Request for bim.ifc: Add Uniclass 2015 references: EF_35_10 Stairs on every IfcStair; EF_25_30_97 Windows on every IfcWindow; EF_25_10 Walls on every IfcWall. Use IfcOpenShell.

First a look at what the model holds.

```python
import ifcopenshell

model = ifcopenshell.open("bim.ifc")
print(model.schema)
print("classifications:", [c.Name for c in model.by_type("IfcClassification")])
for ifc_class in ("IfcDoor", "IfcRoof", "IfcStair", "IfcWall", "IfcWindow"):
    print(ifc_class, len(model.by_type(ifc_class)))
```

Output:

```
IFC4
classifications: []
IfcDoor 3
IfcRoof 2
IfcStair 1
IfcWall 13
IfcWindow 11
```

```python
import ifcopenshell
import ifcopenshell.api.classification

model = ifcopenshell.open("bim.ifc")

system = ifcopenshell.api.classification.add_classification(model, classification="Uniclass 2015")

codes = {
    "IfcStair": ("EF_35_10", "Stairs"),
    "IfcWindow": ("EF_25_30_97", "Windows"),
    "IfcWall": ("EF_25_10", "Walls"),
}
for ifc_class, (code, name) in codes.items():
    products = model.by_type(ifc_class)
    ifcopenshell.api.classification.add_reference(
        model, products=products, classification=system, identification=code, name=name
    )
    print(code, len(products))

model.write("bim-out.ifc")
```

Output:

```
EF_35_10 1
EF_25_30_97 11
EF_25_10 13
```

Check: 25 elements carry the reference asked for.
